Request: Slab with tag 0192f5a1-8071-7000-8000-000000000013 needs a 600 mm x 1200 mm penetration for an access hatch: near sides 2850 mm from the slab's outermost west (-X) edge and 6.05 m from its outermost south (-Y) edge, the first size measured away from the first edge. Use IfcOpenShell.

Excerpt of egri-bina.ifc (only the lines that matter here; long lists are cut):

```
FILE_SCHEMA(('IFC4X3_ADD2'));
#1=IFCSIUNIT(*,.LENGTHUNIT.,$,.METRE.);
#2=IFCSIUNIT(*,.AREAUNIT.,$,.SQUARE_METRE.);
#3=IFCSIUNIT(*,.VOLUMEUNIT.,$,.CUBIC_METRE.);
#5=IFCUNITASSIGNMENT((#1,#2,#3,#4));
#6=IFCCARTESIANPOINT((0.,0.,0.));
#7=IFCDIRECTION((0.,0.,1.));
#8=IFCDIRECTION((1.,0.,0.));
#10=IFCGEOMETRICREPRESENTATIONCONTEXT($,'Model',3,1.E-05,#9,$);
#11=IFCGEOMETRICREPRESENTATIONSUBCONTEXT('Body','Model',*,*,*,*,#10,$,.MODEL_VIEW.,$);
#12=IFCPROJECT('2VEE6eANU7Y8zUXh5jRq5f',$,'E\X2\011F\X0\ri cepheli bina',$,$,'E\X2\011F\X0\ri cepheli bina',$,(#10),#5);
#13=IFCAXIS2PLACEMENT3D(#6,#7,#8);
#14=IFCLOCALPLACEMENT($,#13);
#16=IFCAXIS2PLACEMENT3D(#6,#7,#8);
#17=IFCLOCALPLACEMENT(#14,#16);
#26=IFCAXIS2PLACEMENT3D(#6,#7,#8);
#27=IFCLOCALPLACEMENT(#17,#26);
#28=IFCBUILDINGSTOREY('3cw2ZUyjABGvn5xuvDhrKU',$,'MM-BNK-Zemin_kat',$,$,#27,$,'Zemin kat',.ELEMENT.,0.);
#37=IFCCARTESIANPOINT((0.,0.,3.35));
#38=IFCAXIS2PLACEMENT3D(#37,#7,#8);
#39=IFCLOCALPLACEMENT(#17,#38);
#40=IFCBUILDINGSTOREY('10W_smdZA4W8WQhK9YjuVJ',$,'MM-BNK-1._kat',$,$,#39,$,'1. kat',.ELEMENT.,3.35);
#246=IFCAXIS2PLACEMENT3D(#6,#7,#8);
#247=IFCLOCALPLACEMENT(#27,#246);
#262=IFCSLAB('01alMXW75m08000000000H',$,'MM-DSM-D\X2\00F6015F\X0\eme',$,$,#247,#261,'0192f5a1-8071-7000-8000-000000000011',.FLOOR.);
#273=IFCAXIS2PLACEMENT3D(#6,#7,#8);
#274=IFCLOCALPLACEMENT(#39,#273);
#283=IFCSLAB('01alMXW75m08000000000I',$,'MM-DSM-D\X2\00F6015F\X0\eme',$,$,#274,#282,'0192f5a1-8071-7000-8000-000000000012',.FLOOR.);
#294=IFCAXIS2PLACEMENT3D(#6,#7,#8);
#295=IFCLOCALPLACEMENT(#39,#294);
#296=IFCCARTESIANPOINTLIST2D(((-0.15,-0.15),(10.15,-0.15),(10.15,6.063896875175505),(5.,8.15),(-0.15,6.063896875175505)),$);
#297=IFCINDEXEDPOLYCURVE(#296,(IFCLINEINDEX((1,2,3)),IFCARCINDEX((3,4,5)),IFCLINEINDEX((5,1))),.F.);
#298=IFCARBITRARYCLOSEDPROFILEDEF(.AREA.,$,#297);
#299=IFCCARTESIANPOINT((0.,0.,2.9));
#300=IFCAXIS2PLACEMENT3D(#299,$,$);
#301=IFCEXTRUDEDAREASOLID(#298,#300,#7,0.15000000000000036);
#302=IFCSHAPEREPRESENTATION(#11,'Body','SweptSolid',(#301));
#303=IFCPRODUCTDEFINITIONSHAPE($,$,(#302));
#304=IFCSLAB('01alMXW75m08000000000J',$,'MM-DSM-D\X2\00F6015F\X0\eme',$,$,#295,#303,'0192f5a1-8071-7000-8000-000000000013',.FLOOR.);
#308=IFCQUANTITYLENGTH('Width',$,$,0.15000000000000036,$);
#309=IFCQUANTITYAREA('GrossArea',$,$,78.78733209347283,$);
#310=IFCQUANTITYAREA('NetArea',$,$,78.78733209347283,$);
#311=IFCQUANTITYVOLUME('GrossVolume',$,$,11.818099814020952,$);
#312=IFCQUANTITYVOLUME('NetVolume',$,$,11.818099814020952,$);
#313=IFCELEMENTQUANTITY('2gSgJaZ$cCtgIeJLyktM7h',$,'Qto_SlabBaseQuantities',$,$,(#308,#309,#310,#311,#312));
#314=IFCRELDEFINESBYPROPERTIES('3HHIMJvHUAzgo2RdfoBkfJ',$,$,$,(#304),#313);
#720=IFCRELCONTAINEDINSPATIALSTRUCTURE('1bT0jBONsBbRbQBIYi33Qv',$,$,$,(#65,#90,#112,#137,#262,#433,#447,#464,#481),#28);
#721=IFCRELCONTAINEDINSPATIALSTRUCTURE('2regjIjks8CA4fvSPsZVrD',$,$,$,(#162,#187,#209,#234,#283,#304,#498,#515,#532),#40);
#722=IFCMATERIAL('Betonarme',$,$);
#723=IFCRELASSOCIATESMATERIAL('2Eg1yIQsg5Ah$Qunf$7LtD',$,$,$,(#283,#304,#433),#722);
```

```python
import numpy as np
import ifcopenshell
import ifcopenshell.api.feature
import ifcopenshell.api.geometry
import ifcopenshell.api.pset
import ifcopenshell.api.root
import ifcopenshell.geom
import ifcopenshell.util.element
import ifcopenshell.util.placement
import ifcopenshell.util.representation
import ifcopenshell.util.shape
import ifcopenshell.util.unit

model = ifcopenshell.open("egri-bina.ifc")
unit_scale = ifcopenshell.util.unit.calculate_unit_scale(model)
area_scale = ifcopenshell.util.unit.calculate_unit_scale(model, "AREAUNIT")
volume_scale = ifcopenshell.util.unit.calculate_unit_scale(model, "VOLUMEUNIT")
settings = ifcopenshell.geom.settings()


def volume(element):
    """Net volume in cubic metres, openings subtracted."""
    shape = ifcopenshell.geom.create_shape(settings, element)
    return ifcopenshell.util.shape.get_volume(shape.geometry)


slab = model.by_id(304)
before = volume(slab)

# Extent in the slab's own axes, in metres. The edges named are its -X and -Y sides.
slab_shape = ifcopenshell.geom.create_shape(settings, slab)
vertices = ifcopenshell.util.shape.get_vertices(slab_shape.geometry)
x_min, y_min, bottom = vertices.min(axis=0)
top = vertices[:, 2].max()

opening = ifcopenshell.api.root.create_entity(model, ifc_class="IfcOpeningElement", name="Access hatch opening", predefined_type="OPENING")
context = ifcopenshell.util.representation.get_context(model, "Model", "Body", "MODEL_VIEW")
width, depth = 0.6, 1.2
outline = [(0.0, 0.0), (width, 0.0), (width, depth), (0.0, depth), (0.0, 0.0)]
# Overshoot both faces by 50 mm so the cut is clean.
shape = ifcopenshell.api.geometry.add_slab_representation(
    model, context=context, depth=top - bottom + 0.1, polyline=outline
)
ifcopenshell.api.geometry.assign_representation(model, product=opening, representation=shape)

matrix = ifcopenshell.util.placement.get_local_placement(slab.ObjectPlacement)
matrix[:, 3] = matrix @ np.append(np.array([x_min + 2.85, y_min + 6.05, bottom - 0.05]) / unit_scale, 1.0)
ifcopenshell.api.geometry.edit_object_placement(model, product=opening, matrix=matrix, is_si=False)
ifcopenshell.api.feature.add_feature(model, feature=opening, element=slab)

after = volume(slab)

# Update the slab's stored quantities.
qto = model.by_id(ifcopenshell.util.element.get_pset(slab, "Qto_SlabBaseQuantities", should_inherit=False)["id"])
ifcopenshell.api.pset.edit_qto(model, qto=qto, properties={
    "NetArea": after / (top - bottom) / area_scale,
    "NetVolume": after / volume_scale,
})

print(f"slab volume {before:.3f} -> {after:.3f} m3")

model.write("egri-bina-out.ifc")
```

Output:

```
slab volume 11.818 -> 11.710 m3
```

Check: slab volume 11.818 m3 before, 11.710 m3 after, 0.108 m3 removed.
